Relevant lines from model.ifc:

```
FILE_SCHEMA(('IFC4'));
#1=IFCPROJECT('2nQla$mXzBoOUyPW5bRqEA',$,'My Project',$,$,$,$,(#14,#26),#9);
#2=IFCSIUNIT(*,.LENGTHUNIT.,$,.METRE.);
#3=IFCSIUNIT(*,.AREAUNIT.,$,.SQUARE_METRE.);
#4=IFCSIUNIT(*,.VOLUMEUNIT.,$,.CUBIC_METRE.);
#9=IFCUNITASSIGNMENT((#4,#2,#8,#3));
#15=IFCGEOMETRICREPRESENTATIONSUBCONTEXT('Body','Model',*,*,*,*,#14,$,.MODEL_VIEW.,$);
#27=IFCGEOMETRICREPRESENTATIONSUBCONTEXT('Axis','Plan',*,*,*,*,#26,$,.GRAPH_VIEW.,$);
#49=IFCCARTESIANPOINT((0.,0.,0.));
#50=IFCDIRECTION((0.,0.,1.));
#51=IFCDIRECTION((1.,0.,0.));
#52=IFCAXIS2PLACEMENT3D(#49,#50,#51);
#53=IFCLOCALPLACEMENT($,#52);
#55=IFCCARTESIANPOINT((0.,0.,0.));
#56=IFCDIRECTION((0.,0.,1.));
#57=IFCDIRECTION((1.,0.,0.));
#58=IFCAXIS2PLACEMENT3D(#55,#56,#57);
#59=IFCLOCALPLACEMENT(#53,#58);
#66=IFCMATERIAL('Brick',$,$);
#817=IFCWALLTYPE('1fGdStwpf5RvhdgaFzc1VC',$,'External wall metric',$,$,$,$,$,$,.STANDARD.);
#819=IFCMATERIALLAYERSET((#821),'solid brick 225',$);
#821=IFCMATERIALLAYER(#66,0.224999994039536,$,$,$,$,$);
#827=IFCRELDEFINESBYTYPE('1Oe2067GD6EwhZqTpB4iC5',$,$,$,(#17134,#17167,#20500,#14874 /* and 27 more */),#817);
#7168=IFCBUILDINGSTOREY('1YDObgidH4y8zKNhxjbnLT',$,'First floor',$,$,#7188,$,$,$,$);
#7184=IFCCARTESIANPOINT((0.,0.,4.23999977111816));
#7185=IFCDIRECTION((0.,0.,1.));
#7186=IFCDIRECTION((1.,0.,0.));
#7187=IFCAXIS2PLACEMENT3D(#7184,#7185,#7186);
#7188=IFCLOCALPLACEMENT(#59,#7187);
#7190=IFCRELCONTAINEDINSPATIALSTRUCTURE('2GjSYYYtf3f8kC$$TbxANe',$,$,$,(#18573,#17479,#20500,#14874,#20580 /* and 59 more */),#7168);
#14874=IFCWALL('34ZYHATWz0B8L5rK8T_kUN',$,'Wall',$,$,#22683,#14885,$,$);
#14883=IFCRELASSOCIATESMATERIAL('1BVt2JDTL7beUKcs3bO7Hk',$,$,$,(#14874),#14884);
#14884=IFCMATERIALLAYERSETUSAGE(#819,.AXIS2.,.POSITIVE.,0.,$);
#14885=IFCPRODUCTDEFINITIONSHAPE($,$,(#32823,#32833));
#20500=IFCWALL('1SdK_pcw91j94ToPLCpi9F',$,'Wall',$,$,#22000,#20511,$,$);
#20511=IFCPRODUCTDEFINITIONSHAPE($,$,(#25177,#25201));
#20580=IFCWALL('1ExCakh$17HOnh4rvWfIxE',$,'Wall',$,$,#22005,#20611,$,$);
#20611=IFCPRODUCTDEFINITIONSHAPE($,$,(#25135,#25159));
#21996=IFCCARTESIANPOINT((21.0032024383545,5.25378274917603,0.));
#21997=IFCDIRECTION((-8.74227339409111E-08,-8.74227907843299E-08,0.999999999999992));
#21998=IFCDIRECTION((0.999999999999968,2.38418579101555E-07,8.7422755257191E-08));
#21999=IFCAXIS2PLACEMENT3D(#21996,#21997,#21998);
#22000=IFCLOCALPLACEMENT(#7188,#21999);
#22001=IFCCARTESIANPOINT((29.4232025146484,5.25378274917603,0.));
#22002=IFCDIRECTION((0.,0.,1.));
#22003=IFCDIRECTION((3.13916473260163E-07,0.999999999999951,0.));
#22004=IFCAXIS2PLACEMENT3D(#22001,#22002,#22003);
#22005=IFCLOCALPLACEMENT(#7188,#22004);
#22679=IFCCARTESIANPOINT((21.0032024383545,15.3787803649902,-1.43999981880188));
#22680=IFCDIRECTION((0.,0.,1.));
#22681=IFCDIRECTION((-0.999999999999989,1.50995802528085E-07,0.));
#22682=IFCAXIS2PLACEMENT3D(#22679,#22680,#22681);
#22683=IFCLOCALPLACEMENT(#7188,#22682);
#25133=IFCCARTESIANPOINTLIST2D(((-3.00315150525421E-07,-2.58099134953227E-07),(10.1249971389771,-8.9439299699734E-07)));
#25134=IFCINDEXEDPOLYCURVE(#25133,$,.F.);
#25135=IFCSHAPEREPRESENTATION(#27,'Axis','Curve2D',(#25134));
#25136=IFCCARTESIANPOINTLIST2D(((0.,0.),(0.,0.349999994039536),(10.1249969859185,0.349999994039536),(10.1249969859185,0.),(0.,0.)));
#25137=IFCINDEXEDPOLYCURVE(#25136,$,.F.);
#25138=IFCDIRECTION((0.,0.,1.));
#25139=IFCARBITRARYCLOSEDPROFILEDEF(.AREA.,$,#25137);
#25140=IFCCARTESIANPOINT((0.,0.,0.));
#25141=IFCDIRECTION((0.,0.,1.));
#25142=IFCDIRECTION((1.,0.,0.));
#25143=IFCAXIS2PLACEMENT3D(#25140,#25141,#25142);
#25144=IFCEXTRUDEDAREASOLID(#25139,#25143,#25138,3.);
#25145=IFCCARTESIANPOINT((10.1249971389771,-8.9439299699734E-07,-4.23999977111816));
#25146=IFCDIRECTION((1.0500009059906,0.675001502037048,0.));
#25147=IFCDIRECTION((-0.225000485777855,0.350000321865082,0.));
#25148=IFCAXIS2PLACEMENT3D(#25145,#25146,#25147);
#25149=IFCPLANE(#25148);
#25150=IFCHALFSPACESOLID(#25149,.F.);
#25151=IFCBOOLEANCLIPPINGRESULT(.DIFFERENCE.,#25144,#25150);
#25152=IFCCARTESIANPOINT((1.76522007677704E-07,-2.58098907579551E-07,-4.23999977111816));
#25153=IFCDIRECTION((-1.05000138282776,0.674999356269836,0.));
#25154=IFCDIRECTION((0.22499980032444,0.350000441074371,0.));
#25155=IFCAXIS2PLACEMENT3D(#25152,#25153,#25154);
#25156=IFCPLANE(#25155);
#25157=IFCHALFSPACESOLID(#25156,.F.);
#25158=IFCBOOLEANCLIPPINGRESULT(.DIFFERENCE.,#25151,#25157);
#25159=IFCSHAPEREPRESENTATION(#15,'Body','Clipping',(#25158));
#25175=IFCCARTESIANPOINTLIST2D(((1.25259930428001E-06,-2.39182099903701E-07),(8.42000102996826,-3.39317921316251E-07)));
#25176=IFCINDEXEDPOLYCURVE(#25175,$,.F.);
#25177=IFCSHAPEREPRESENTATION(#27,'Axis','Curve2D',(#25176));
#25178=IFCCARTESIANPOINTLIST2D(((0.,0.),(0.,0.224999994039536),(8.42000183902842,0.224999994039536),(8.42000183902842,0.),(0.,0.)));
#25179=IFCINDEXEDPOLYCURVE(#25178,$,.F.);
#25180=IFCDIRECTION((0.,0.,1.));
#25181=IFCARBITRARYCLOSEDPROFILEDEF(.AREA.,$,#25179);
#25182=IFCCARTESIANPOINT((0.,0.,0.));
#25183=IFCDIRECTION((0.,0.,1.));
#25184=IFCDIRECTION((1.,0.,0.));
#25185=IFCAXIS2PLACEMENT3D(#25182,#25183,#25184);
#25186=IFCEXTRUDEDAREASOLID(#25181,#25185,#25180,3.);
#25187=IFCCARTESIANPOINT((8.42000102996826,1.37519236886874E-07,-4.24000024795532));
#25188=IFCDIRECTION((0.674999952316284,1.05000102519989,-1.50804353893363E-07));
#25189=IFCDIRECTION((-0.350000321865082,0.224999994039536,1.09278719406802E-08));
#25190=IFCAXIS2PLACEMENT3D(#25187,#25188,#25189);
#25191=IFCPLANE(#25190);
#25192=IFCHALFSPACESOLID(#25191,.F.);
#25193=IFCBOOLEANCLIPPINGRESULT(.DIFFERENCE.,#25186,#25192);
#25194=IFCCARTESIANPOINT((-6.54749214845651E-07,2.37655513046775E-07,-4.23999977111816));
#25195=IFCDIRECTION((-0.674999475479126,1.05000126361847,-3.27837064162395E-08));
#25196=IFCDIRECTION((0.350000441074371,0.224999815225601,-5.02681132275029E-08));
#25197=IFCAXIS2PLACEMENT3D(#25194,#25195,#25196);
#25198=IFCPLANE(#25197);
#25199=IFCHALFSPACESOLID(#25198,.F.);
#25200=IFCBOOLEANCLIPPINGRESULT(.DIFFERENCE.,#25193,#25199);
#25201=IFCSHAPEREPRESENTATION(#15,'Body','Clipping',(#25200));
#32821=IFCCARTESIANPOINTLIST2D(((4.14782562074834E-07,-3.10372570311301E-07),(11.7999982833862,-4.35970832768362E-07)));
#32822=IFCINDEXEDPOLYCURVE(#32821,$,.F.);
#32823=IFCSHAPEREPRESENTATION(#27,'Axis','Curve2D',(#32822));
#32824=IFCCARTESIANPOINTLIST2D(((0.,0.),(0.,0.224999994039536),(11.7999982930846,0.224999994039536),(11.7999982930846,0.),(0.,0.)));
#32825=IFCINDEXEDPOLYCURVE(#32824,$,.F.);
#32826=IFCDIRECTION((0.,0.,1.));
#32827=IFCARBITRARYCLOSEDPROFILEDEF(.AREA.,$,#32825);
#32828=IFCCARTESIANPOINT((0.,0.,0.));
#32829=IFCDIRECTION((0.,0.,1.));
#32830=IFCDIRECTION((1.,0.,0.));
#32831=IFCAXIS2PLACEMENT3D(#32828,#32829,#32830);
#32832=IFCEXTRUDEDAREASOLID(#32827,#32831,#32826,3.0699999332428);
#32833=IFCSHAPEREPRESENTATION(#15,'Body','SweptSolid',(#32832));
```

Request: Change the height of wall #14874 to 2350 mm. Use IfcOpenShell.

```python
import ifcopenshell
import ifcopenshell.geom
import ifcopenshell.util.representation
import ifcopenshell.util.shape

model = ifcopenshell.open("model.ifc")
settings = ifcopenshell.geom.settings()


def volume(element):
    """Net volume in cubic metres, openings subtracted."""
    shape = ifcopenshell.geom.create_shape(settings, element)
    return ifcopenshell.util.shape.get_volume(shape.geometry)


wall = model.by_guid("34ZYHATWz0B8L5rK8T_kUN")
before = volume(wall)

body = ifcopenshell.util.representation.get_representation(wall, "Model", "Body")
solid = body.Items[0]
old_height = solid.Depth
solid.Depth = 2.35
after = volume(wall)

print(f"height {old_height:g} -> {solid.Depth:g}, volume {before:.3f} -> {after:.3f} m3")

model.write("model_edited.ifc")
```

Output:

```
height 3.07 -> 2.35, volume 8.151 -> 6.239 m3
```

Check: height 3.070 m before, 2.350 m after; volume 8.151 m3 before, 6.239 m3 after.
